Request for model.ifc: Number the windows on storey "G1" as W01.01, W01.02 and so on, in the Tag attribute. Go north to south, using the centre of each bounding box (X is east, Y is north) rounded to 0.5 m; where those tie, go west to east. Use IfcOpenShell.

First a look at what the model holds.

```python
import ifcopenshell
import ifcopenshell.util.element
import ifcopenshell.util.placement

model = ifcopenshell.open("model.ifc")
print(model.schema)
storey = next(s for s in model.by_type("IfcBuildingStorey") if s.Name == "G1")
windows = [e for e in ifcopenshell.util.element.get_decomposition(storey) if e.is_a("IfcWindow")]
for e in sorted(windows, key=lambda e: e.id()):
    origin = ifcopenshell.util.placement.get_local_placement(e.ObjectPlacement)[:3, 3]
    print(e.id(), e.Tag, e.Name, origin.round(2) + 0.0, sep=" | ")
```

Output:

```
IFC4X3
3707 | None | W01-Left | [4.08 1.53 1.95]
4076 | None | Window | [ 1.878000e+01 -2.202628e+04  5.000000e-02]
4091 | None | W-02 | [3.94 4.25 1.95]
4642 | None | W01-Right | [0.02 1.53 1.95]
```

```python
import ifcopenshell
import ifcopenshell.geom
import ifcopenshell.util.element
import ifcopenshell.util.shape

model = ifcopenshell.open("model.ifc")
settings = ifcopenshell.geom.settings()
settings.set("use-world-coords", True)


def centre(element):
    shape = ifcopenshell.geom.create_shape(settings, element)
    return ifcopenshell.util.shape.get_bbox_centroid(shape.geometry)


storey = next(s for s in model.by_type("IfcBuildingStorey") if s.Name == "G1")
windows = [e for e in ifcopenshell.util.element.get_decomposition(storey) if e.is_a("IfcWindow")]

# Insertion points can sit at a corner or the storey origin, so sort by the geometry (in metres).
centres = {e: centre(e) for e in windows}
windows.sort(key=lambda e: (-round(centres[e][1] / 0.5), centres[e][0]))

for i, e in enumerate(windows, start=1):
    number = f"W01.{i:02d}"
    e.Tag = number
    print(e.id(), number)

model.write("model-out.ifc")
```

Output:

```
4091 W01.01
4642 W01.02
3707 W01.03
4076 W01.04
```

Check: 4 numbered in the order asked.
